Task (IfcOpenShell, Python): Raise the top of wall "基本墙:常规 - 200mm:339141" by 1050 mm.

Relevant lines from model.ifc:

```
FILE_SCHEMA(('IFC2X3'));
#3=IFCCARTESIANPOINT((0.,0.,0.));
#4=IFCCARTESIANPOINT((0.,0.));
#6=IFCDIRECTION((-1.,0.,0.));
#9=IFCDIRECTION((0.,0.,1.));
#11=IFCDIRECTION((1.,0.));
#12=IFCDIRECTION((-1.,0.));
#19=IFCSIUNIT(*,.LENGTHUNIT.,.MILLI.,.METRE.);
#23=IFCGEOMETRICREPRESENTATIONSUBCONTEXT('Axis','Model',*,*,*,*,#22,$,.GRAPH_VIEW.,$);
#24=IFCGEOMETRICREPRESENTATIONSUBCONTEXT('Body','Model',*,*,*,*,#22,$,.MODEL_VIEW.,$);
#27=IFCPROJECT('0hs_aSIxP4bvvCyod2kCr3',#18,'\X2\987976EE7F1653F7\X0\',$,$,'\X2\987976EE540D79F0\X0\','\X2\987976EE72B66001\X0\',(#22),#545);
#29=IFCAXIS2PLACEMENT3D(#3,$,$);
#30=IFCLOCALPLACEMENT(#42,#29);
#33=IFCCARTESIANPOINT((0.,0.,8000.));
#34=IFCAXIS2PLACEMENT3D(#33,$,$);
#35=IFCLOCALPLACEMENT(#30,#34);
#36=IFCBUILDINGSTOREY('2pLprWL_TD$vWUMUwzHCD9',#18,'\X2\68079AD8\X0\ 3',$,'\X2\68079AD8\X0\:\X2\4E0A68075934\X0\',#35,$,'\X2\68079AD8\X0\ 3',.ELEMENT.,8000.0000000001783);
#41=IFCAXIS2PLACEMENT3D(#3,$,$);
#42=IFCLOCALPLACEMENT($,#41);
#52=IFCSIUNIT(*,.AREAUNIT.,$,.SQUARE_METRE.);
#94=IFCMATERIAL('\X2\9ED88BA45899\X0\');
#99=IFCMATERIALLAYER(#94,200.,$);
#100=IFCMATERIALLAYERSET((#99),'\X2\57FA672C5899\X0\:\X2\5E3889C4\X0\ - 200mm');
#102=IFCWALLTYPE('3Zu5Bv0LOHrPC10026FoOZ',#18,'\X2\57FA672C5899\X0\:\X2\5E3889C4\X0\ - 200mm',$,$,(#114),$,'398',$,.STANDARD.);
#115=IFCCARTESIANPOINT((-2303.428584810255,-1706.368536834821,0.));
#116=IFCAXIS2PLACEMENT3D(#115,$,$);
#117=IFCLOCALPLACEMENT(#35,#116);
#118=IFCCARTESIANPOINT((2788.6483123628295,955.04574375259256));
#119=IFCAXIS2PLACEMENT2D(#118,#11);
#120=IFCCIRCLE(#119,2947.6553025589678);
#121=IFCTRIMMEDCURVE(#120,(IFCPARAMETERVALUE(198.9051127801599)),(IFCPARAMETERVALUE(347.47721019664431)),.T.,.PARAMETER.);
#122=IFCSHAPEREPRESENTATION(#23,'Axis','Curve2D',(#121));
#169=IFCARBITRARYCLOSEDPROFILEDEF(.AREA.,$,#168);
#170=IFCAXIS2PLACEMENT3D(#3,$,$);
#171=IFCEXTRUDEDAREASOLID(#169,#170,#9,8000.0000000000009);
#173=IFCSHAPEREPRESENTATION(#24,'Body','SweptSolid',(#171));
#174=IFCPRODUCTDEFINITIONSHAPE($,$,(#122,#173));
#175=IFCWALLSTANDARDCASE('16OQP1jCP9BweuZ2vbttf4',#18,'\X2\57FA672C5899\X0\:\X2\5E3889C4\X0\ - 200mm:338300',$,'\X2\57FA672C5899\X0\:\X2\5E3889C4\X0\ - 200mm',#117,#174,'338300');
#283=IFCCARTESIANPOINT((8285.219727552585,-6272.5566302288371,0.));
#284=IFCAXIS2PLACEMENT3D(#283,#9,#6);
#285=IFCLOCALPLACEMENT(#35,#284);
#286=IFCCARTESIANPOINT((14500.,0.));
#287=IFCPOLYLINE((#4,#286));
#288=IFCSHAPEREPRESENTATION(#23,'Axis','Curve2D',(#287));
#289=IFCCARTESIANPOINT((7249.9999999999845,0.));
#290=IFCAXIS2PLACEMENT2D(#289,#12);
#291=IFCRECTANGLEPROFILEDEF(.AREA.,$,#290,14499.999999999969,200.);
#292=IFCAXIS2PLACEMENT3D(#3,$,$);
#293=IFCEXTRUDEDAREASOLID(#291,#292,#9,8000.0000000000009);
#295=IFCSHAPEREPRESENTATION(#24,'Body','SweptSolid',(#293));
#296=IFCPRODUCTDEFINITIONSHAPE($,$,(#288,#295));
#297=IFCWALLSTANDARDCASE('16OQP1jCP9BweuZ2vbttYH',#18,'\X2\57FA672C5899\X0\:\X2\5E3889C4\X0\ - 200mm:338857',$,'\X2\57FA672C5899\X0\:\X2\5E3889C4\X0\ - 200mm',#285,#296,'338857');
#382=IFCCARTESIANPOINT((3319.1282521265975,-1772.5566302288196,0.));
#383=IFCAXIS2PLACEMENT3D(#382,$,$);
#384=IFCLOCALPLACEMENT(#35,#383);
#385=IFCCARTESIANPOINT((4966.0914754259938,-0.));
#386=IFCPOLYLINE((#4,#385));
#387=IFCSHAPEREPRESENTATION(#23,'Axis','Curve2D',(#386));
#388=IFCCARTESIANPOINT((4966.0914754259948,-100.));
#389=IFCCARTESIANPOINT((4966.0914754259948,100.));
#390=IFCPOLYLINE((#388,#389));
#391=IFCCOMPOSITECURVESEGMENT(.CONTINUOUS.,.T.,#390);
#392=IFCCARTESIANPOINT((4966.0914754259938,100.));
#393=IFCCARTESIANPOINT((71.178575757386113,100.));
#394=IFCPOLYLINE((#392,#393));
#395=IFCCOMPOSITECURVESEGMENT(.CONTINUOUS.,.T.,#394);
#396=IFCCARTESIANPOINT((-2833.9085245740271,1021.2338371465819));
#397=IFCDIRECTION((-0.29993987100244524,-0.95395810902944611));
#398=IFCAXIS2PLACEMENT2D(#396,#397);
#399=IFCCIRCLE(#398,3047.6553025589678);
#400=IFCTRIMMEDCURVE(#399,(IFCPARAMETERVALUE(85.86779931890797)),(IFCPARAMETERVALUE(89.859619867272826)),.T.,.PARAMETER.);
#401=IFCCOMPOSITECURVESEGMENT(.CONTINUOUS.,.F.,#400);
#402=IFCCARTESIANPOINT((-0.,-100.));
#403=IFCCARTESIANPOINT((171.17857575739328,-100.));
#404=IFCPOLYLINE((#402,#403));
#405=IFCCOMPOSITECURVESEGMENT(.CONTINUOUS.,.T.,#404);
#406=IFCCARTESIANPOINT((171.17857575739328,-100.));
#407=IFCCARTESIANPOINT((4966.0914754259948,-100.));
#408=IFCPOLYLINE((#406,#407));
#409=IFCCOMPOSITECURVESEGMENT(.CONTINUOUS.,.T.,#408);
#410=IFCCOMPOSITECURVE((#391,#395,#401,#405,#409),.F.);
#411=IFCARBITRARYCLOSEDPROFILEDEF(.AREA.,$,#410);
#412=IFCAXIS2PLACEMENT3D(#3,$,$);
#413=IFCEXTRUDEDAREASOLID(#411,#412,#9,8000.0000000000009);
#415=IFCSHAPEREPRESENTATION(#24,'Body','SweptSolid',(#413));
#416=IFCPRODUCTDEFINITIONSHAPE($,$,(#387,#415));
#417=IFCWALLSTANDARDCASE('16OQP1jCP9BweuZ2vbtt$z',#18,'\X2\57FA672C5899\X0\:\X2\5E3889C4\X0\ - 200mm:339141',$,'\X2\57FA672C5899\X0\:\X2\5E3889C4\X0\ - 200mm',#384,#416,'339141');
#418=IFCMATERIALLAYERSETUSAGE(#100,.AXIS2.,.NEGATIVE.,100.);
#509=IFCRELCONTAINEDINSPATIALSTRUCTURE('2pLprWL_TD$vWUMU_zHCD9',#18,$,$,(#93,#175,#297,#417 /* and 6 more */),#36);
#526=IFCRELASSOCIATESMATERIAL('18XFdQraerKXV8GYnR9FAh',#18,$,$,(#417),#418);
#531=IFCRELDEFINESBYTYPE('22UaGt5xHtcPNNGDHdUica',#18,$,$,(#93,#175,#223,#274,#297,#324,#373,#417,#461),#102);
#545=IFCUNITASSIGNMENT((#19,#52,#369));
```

```python
import ifcopenshell
import ifcopenshell.geom
import ifcopenshell.util.representation
import ifcopenshell.util.shape

model = ifcopenshell.open("model.ifc")
settings = ifcopenshell.geom.settings()


def volume(element):
    """Net volume in cubic metres, openings subtracted."""
    shape = ifcopenshell.geom.create_shape(settings, element)
    return ifcopenshell.util.shape.get_volume(shape.geometry)


wall = model.by_guid("16OQP1jCP9BweuZ2vbtt$z")
before = volume(wall)

body = ifcopenshell.util.representation.get_representation(wall, "Model", "Body")
solid = body.Items[0]
old_height = solid.Depth
solid.Depth += 1050.0
after = volume(wall)

print(f"height {old_height:g} -> {solid.Depth:g}, volume {before:.3f} -> {after:.3f} m3")

model.write("model_edited.ifc")
```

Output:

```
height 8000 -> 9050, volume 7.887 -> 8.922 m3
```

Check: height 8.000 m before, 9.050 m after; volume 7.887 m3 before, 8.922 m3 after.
